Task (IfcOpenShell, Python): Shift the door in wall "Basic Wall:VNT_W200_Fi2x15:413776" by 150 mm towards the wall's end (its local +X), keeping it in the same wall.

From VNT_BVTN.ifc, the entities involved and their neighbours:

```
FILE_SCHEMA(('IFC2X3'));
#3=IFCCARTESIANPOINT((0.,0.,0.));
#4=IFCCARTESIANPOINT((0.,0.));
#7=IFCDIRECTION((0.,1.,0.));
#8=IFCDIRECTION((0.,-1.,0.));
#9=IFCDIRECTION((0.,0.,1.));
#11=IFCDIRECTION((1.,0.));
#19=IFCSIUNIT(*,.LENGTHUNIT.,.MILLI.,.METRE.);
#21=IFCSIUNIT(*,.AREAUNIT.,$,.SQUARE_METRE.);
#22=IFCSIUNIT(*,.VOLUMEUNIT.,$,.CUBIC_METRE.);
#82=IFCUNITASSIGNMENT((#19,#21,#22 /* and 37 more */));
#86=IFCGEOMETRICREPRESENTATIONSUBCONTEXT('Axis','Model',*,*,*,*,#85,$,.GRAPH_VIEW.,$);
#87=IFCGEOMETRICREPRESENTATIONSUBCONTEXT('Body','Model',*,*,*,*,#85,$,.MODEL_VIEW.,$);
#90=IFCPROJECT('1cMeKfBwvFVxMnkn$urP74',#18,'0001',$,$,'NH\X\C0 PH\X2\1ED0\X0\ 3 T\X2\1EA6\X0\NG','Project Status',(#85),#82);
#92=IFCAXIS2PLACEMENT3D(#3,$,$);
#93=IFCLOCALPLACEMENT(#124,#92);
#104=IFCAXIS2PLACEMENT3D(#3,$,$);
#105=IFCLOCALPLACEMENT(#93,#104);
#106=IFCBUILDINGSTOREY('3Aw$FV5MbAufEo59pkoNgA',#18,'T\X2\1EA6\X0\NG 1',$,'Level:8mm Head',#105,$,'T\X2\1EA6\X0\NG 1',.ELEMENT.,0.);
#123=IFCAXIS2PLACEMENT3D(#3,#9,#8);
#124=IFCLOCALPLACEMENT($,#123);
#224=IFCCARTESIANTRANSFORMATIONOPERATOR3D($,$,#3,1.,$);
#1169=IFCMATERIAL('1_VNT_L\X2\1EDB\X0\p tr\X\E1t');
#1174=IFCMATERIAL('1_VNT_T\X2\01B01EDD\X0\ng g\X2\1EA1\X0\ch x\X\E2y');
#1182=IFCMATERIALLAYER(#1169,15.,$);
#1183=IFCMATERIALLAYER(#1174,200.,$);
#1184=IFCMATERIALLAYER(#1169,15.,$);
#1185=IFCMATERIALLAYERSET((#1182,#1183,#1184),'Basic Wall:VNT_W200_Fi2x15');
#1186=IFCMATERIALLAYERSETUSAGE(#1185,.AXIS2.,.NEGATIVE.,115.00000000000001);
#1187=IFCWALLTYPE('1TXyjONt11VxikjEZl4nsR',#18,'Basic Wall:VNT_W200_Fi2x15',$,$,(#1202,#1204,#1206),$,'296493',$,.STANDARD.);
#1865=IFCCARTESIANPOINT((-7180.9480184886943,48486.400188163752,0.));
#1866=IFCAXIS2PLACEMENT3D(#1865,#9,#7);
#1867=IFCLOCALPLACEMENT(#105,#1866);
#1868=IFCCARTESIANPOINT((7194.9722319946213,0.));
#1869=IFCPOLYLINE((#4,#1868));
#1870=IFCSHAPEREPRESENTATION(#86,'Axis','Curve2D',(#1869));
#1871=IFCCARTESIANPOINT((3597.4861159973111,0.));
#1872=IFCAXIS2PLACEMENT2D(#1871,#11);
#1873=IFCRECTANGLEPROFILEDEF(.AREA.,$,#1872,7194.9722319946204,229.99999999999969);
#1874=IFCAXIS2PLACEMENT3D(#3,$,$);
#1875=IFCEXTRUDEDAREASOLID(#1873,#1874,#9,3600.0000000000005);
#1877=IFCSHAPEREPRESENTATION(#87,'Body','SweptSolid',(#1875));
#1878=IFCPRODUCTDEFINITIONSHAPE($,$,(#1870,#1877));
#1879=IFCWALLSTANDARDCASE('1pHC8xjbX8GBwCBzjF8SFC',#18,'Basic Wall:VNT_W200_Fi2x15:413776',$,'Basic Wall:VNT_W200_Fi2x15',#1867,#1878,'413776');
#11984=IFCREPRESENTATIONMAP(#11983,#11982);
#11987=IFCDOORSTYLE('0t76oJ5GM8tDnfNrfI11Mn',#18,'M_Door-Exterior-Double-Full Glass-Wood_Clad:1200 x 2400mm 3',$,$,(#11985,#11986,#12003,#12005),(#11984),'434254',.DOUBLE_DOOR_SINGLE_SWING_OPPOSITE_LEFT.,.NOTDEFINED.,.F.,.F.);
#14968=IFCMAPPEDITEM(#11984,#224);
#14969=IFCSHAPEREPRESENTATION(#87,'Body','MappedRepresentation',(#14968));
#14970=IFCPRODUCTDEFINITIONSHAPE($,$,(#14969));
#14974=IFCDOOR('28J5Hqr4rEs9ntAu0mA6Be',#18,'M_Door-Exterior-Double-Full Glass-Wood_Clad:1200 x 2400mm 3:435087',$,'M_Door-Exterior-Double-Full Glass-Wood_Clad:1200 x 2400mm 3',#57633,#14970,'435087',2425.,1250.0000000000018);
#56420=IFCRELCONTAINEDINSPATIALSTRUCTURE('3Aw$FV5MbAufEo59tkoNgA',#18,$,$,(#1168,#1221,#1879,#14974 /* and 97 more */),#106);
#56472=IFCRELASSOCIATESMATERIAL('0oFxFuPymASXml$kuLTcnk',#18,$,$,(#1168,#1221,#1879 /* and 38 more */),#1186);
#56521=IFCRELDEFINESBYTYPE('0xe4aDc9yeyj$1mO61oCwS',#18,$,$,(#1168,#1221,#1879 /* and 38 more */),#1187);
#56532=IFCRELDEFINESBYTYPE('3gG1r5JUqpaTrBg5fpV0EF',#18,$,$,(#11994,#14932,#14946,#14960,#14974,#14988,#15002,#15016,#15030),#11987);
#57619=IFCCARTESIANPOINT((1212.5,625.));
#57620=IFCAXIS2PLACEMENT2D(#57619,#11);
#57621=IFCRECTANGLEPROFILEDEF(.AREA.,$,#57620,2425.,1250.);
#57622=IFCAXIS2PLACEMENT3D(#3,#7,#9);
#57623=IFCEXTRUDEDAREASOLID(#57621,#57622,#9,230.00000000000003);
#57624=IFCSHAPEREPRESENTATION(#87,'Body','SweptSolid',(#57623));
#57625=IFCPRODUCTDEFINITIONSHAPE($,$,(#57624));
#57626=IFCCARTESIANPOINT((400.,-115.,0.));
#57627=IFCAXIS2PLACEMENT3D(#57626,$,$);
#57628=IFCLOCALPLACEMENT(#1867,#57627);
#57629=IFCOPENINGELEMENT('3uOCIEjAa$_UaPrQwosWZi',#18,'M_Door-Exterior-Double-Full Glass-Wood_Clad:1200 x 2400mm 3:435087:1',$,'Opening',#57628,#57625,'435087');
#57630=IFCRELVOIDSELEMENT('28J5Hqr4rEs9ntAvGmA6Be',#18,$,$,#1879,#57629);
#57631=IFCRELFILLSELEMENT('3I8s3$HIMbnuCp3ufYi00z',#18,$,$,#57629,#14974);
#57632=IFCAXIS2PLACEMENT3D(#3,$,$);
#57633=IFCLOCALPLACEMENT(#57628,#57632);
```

```python
import ifcopenshell
import ifcopenshell.api.geometry
import ifcopenshell.util.placement

model = ifcopenshell.open("VNT_BVTN.ifc")

door = model.by_guid("28J5Hqr4rEs9ntAu0mA6Be")
opening = door.FillsVoids[0].RelatingOpeningElement
wall = opening.VoidsElements[0].RelatingBuildingElement

wall_matrix = ifcopenshell.util.placement.get_local_placement(wall.ObjectPlacement)
shift = wall_matrix[:3, 0] * 150.0
before = ifcopenshell.util.placement.get_local_placement(door.ObjectPlacement)[:3, 3].copy()

# The door is placed relative to its opening, so it follows when the opening moves.
matrix = ifcopenshell.util.placement.get_local_placement(opening.ObjectPlacement)
matrix[:3, 3] += shift
ifcopenshell.api.geometry.edit_object_placement(
    model, product=opening, matrix=matrix, is_si=False, should_transform_children=True
)

after = ifcopenshell.util.placement.get_local_placement(door.ObjectPlacement)[:3, 3]
print("door moved by", (after - before).round(3) + 0.0)

model.write("VNT_BVTN_updated.ifc")
```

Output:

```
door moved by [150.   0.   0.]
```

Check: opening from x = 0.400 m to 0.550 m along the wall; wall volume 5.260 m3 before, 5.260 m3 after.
